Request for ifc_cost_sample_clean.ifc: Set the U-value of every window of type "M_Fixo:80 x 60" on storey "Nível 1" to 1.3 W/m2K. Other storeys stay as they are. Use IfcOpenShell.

First a look at what the model holds.

```python
import ifcopenshell
import ifcopenshell.util.element

model = ifcopenshell.open("ifc_cost_sample_clean.ifc")
print(model.schema)
storey = next(s for s in model.by_type("IfcBuildingStorey") if s.Name == "Nível 1")
windows = [e for e in ifcopenshell.util.element.get_decomposition(storey) if e.is_a("IfcWindow")]
seen = {}
for e in windows:
    element_type = ifcopenshell.util.element.get_type(e)
    key = (element_type.Name if element_type != e and element_type else None, ifcopenshell.util.element.get_pset(e, "Pset_WindowCommon", "ThermalTransmittance"))
    seen[key] = seen.get(key, 0) + 1
for (name, value), count in sorted(seen.items(), key=str):
    print(count, "x", name, "|", value)
```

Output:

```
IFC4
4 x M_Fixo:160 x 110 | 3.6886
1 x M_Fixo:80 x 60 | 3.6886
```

```python
import ifcopenshell
import ifcopenshell.api.pset
import ifcopenshell.util.element

model = ifcopenshell.open("ifc_cost_sample_clean.ifc")

storey = next(s for s in model.by_type("IfcBuildingStorey") if s.Name == "Nível 1")
windows = [e for e in ifcopenshell.util.element.get_decomposition(storey) if e.is_a("IfcWindow")]

count = 0
for e in windows:
    element_type = ifcopenshell.util.element.get_type(e)
    if element_type in (None, e) or element_type.Name != "M_Fixo:80 x 60":
        continue
    # add_pset returns the element's existing set when there is one.
    pset = ifcopenshell.api.pset.add_pset(model, product=e, name="Pset_WindowCommon")
    ifcopenshell.api.pset.edit_pset(model, pset=pset, properties={"ThermalTransmittance": 1.3})
    count += 1

print(count, "windows updated")

model.write("ifc_cost_sample_clean_v2.ifc")
```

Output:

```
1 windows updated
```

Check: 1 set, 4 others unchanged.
